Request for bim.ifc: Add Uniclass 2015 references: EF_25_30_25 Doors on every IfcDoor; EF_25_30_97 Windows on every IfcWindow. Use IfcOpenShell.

First a look at what the model holds.

```python
import ifcopenshell

model = ifcopenshell.open("bim.ifc")
print(model.schema)
print("classifications:", [c.Name for c in model.by_type("IfcClassification")])
for ifc_class in ("IfcDoor", "IfcRoof", "IfcStair", "IfcWall", "IfcWindow"):
    print(ifc_class, len(model.by_type(ifc_class)))
```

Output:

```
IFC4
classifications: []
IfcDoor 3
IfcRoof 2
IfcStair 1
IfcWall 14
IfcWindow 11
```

```python
import ifcopenshell
import ifcopenshell.api.classification

model = ifcopenshell.open("bim.ifc")

system = ifcopenshell.api.classification.add_classification(model, classification="Uniclass 2015")

codes = {
    "IfcDoor": ("EF_25_30_25", "Doors"),
    "IfcWindow": ("EF_25_30_97", "Windows"),
}
for ifc_class, (code, name) in codes.items():
    products = model.by_type(ifc_class)
    ifcopenshell.api.classification.add_reference(
        model, products=products, classification=system, identification=code, name=name
    )
    print(code, len(products))

model.write("bim_rev.ifc")
```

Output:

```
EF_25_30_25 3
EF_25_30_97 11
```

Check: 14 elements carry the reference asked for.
